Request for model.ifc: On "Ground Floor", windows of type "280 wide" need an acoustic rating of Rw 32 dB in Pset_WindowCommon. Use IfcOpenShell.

First a look at what the model holds.

```python
import ifcopenshell
import ifcopenshell.util.element

model = ifcopenshell.open("model.ifc")
print(model.schema)
storey = next(s for s in model.by_type("IfcBuildingStorey") if s.Name == "Ground Floor")
windows = [e for e in ifcopenshell.util.element.get_decomposition(storey) if e.is_a("IfcWindow")]
seen = {}
for e in windows:
    element_type = ifcopenshell.util.element.get_type(e)
    key = (element_type.Name if element_type != e and element_type else None, ifcopenshell.util.element.get_pset(e, "Pset_WindowCommon", "AcousticRating"))
    seen[key] = seen.get(key, 0) + 1
for (name, value), count in sorted(seen.items(), key=str):
    print(count, "x", name, "|", value)
```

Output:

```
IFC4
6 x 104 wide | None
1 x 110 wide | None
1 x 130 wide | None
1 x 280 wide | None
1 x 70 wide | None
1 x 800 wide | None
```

```python
import ifcopenshell
import ifcopenshell.api.pset
import ifcopenshell.util.element

model = ifcopenshell.open("model.ifc")

storey = next(s for s in model.by_type("IfcBuildingStorey") if s.Name == "Ground Floor")
windows = [e for e in ifcopenshell.util.element.get_decomposition(storey) if e.is_a("IfcWindow")]

count = 0
for e in windows:
    element_type = ifcopenshell.util.element.get_type(e)
    if element_type in (None, e) or element_type.Name != "280 wide":
        continue
    # add_pset returns the element's existing set when there is one.
    pset = ifcopenshell.api.pset.add_pset(model, product=e, name="Pset_WindowCommon")
    ifcopenshell.api.pset.edit_pset(model, pset=pset, properties={"AcousticRating": "Rw 32 dB"})
    count += 1

print(count, "windows updated")

model.write("model_v2.ifc")
```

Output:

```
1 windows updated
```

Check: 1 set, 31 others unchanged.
